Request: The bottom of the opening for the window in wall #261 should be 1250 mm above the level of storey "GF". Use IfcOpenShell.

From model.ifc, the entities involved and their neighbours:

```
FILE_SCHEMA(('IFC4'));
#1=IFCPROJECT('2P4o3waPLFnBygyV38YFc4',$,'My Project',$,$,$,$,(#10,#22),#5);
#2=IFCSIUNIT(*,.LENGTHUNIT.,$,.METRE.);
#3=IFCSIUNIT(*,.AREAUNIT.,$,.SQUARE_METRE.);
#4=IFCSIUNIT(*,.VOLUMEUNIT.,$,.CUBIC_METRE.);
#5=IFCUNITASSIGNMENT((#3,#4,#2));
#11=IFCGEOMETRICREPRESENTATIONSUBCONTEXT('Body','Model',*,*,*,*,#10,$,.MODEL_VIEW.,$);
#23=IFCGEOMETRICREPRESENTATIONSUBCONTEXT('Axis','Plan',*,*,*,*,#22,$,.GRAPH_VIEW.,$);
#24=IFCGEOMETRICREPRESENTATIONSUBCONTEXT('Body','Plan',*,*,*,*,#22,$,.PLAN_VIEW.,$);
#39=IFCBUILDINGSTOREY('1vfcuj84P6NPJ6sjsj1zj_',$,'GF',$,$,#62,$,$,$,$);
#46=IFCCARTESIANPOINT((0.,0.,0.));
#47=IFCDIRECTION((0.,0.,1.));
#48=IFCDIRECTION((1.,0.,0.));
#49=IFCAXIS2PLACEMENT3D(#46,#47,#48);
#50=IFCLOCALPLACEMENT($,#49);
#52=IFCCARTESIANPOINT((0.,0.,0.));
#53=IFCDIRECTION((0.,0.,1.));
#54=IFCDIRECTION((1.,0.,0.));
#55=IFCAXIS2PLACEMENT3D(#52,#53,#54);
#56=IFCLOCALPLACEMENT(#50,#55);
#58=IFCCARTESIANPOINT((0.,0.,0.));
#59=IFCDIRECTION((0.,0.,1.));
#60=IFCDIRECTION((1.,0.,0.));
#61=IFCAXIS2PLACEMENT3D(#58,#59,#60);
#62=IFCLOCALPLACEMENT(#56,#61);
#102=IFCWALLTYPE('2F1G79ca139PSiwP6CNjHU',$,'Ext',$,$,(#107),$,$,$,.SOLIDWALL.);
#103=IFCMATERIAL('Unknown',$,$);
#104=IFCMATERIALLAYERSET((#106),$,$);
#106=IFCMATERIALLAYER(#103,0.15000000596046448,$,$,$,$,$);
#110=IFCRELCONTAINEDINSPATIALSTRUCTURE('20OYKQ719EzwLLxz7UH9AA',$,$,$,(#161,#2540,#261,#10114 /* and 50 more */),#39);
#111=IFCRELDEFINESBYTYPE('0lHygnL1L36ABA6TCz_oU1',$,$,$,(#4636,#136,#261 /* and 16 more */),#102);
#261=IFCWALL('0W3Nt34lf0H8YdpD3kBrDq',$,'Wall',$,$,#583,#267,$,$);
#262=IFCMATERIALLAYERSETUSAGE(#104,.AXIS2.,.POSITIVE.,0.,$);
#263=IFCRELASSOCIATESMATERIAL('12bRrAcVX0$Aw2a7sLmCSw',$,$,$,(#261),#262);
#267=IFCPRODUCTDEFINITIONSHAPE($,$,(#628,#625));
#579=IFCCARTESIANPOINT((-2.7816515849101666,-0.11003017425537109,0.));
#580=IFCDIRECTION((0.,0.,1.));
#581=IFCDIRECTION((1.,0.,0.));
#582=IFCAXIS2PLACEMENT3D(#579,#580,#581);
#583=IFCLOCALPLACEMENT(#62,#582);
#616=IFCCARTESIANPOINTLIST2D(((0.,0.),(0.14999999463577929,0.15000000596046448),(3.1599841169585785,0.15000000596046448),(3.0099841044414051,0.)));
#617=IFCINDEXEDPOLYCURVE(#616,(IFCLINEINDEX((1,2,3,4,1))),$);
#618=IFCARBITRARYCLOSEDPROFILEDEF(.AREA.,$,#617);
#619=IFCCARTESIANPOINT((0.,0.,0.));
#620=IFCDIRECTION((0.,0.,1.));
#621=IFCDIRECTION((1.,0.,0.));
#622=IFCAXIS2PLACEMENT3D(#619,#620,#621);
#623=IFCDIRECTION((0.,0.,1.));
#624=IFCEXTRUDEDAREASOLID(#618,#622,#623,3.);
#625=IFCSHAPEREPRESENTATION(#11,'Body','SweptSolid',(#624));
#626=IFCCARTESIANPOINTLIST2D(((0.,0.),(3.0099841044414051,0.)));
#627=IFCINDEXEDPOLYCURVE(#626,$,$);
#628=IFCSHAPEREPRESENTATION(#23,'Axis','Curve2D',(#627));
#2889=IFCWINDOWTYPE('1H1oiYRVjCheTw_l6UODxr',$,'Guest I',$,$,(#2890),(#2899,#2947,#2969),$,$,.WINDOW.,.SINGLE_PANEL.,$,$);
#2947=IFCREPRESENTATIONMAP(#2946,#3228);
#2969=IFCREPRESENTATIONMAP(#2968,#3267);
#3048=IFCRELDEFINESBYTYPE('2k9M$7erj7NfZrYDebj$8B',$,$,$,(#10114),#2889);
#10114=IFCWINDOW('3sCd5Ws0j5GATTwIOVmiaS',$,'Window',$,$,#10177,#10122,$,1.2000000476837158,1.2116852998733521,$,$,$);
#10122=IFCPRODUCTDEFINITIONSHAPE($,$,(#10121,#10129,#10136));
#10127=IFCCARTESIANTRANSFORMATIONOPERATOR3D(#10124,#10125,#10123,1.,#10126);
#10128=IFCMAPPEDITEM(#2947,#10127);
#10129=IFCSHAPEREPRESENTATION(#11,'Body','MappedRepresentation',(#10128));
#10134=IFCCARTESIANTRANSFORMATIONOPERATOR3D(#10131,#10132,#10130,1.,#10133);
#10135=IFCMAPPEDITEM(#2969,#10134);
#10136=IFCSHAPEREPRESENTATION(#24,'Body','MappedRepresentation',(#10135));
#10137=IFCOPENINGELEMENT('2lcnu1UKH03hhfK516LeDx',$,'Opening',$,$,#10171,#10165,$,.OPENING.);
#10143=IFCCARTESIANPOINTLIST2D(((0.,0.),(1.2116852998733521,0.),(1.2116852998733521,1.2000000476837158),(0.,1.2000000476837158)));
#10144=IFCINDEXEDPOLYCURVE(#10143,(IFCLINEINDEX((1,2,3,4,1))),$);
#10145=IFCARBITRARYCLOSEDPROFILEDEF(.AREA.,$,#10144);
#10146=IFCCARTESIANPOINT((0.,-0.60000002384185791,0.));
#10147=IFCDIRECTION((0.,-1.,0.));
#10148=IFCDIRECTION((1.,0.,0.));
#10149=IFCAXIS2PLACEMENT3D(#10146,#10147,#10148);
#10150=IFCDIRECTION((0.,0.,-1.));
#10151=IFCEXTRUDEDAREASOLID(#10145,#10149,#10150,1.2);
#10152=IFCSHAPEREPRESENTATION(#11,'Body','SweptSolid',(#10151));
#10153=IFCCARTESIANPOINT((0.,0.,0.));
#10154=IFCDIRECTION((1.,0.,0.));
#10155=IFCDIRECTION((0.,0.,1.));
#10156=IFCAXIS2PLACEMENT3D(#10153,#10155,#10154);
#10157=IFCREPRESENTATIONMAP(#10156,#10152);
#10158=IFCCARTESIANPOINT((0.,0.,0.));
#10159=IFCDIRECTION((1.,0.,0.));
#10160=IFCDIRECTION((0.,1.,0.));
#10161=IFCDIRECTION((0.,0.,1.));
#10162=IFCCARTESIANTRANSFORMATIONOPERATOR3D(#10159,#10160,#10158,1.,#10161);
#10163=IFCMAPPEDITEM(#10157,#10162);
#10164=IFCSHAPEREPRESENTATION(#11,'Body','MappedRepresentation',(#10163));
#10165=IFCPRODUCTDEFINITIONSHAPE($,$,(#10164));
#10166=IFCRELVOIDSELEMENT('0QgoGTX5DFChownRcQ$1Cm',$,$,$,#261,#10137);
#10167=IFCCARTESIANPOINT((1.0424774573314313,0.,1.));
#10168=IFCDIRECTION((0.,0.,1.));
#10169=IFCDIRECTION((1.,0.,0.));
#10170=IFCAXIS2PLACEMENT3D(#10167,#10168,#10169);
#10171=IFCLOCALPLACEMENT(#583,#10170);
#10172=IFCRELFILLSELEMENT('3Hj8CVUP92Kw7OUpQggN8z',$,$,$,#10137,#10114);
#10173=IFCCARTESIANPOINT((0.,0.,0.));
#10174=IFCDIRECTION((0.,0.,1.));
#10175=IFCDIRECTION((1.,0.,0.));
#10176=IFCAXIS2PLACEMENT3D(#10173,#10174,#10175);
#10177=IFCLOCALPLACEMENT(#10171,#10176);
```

```python
import numpy as np
import ifcopenshell
import ifcopenshell.api.geometry
import ifcopenshell.geom
import ifcopenshell.util.element
import ifcopenshell.util.placement
import ifcopenshell.util.shape
import ifcopenshell.util.unit

model = ifcopenshell.open("model.ifc")
unit_scale = ifcopenshell.util.unit.calculate_unit_scale(model)

window = model.by_guid("3sCd5Ws0j5GATTwIOVmiaS")
opening = window.FillsVoids[0].RelatingOpeningElement
storey = ifcopenshell.util.element.get_container(window, ifc_class="IfcBuildingStorey")
level = ifcopenshell.util.placement.get_local_placement(storey.ObjectPlacement)[2, 3]

# The opening's origin need not be at the sill, so measure its lowest point.
shape = ifcopenshell.geom.create_shape(ifcopenshell.geom.settings(), opening)
bottom = ifcopenshell.util.shape.get_shape_bottom_elevation(shape, shape.geometry) / unit_scale
dz = level + 1.25 / unit_scale - bottom

shift = np.array([0.0, 0.0, dz])
# The window is placed relative to its opening, so it follows when the opening moves.
matrix = ifcopenshell.util.placement.get_local_placement(opening.ObjectPlacement)
matrix[:3, 3] += shift
ifcopenshell.api.geometry.edit_object_placement(
    model, product=opening, matrix=matrix, is_si=False, should_transform_children=True
)

print(f"moved by {dz * unit_scale:+.3f} m")

model.write("model_rev.ifc")
```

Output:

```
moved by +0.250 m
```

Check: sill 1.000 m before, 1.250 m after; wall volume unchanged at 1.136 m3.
